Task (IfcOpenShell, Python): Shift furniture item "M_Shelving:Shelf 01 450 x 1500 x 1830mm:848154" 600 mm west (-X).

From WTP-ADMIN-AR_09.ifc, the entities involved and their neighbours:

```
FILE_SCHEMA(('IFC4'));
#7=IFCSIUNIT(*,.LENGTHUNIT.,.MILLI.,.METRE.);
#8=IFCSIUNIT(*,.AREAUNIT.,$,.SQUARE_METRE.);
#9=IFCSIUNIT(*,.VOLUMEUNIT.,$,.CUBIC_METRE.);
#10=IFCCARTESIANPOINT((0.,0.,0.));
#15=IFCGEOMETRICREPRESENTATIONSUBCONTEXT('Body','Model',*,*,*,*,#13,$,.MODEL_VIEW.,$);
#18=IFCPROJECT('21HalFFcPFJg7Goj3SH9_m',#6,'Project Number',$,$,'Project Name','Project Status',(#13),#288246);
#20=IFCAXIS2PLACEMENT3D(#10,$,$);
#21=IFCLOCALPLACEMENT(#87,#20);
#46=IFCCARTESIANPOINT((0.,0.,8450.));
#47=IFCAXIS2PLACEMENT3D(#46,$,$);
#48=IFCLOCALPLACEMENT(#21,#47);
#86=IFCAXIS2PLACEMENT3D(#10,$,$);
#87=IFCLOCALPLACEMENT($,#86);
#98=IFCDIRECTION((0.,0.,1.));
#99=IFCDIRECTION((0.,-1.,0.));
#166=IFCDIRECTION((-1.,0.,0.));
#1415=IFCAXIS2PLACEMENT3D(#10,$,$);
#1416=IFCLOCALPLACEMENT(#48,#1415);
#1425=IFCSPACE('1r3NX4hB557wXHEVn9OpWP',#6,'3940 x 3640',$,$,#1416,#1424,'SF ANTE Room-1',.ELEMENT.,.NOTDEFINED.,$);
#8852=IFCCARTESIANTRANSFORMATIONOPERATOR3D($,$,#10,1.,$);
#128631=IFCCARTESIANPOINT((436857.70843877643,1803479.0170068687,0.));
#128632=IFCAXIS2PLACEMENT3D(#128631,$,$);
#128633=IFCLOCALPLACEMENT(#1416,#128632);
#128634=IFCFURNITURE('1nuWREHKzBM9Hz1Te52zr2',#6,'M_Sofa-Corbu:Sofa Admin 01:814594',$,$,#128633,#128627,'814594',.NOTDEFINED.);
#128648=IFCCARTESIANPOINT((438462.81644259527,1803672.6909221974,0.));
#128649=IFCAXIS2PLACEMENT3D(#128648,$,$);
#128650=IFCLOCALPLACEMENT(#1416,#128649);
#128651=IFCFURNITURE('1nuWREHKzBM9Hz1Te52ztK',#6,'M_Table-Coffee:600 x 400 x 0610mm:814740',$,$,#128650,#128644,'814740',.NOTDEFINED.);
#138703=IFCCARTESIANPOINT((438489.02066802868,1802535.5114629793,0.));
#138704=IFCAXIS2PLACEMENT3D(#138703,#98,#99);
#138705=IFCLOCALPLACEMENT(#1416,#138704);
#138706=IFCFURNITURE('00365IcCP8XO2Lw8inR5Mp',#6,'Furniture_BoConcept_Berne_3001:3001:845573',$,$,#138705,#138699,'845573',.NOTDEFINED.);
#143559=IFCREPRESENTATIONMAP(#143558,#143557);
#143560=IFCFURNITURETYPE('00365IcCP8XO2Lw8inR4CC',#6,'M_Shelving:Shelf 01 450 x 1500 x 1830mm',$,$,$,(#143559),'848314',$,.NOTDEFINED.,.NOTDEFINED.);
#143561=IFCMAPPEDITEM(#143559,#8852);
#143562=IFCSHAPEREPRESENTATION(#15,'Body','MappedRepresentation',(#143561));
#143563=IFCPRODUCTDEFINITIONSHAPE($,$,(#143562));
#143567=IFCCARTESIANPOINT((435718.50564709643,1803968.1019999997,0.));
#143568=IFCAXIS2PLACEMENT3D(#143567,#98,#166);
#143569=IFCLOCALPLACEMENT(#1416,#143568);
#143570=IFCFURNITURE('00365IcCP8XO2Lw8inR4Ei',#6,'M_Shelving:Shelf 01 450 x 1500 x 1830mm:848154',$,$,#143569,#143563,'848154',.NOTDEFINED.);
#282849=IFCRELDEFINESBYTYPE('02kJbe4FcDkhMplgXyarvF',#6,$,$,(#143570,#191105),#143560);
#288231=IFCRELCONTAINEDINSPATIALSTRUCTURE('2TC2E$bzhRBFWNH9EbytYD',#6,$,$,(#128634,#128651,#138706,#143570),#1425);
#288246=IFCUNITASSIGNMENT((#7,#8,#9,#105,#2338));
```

```python
import ifcopenshell
import ifcopenshell.api.geometry
import ifcopenshell.util.placement
import ifcopenshell.util.unit

model = ifcopenshell.open("WTP-ADMIN-AR_09.ifc")
unit_scale = ifcopenshell.util.unit.calculate_unit_scale(model)

item = model.by_id(143570)
matrix = ifcopenshell.util.placement.get_local_placement(item.ObjectPlacement)
matrix[0, 3] -= 0.6 / unit_scale
ifcopenshell.api.geometry.edit_object_placement(model, product=item, matrix=matrix, is_si=False)

print(ifcopenshell.util.placement.get_local_placement(item.ObjectPlacement).round(3) + 0.0)

model.write("WTP-ADMIN-AR_09_rev.ifc")
```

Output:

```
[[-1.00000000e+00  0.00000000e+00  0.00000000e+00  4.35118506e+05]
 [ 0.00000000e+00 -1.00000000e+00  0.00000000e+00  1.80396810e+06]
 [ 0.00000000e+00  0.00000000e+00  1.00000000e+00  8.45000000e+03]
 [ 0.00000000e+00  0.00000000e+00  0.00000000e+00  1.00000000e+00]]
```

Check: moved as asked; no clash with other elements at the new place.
